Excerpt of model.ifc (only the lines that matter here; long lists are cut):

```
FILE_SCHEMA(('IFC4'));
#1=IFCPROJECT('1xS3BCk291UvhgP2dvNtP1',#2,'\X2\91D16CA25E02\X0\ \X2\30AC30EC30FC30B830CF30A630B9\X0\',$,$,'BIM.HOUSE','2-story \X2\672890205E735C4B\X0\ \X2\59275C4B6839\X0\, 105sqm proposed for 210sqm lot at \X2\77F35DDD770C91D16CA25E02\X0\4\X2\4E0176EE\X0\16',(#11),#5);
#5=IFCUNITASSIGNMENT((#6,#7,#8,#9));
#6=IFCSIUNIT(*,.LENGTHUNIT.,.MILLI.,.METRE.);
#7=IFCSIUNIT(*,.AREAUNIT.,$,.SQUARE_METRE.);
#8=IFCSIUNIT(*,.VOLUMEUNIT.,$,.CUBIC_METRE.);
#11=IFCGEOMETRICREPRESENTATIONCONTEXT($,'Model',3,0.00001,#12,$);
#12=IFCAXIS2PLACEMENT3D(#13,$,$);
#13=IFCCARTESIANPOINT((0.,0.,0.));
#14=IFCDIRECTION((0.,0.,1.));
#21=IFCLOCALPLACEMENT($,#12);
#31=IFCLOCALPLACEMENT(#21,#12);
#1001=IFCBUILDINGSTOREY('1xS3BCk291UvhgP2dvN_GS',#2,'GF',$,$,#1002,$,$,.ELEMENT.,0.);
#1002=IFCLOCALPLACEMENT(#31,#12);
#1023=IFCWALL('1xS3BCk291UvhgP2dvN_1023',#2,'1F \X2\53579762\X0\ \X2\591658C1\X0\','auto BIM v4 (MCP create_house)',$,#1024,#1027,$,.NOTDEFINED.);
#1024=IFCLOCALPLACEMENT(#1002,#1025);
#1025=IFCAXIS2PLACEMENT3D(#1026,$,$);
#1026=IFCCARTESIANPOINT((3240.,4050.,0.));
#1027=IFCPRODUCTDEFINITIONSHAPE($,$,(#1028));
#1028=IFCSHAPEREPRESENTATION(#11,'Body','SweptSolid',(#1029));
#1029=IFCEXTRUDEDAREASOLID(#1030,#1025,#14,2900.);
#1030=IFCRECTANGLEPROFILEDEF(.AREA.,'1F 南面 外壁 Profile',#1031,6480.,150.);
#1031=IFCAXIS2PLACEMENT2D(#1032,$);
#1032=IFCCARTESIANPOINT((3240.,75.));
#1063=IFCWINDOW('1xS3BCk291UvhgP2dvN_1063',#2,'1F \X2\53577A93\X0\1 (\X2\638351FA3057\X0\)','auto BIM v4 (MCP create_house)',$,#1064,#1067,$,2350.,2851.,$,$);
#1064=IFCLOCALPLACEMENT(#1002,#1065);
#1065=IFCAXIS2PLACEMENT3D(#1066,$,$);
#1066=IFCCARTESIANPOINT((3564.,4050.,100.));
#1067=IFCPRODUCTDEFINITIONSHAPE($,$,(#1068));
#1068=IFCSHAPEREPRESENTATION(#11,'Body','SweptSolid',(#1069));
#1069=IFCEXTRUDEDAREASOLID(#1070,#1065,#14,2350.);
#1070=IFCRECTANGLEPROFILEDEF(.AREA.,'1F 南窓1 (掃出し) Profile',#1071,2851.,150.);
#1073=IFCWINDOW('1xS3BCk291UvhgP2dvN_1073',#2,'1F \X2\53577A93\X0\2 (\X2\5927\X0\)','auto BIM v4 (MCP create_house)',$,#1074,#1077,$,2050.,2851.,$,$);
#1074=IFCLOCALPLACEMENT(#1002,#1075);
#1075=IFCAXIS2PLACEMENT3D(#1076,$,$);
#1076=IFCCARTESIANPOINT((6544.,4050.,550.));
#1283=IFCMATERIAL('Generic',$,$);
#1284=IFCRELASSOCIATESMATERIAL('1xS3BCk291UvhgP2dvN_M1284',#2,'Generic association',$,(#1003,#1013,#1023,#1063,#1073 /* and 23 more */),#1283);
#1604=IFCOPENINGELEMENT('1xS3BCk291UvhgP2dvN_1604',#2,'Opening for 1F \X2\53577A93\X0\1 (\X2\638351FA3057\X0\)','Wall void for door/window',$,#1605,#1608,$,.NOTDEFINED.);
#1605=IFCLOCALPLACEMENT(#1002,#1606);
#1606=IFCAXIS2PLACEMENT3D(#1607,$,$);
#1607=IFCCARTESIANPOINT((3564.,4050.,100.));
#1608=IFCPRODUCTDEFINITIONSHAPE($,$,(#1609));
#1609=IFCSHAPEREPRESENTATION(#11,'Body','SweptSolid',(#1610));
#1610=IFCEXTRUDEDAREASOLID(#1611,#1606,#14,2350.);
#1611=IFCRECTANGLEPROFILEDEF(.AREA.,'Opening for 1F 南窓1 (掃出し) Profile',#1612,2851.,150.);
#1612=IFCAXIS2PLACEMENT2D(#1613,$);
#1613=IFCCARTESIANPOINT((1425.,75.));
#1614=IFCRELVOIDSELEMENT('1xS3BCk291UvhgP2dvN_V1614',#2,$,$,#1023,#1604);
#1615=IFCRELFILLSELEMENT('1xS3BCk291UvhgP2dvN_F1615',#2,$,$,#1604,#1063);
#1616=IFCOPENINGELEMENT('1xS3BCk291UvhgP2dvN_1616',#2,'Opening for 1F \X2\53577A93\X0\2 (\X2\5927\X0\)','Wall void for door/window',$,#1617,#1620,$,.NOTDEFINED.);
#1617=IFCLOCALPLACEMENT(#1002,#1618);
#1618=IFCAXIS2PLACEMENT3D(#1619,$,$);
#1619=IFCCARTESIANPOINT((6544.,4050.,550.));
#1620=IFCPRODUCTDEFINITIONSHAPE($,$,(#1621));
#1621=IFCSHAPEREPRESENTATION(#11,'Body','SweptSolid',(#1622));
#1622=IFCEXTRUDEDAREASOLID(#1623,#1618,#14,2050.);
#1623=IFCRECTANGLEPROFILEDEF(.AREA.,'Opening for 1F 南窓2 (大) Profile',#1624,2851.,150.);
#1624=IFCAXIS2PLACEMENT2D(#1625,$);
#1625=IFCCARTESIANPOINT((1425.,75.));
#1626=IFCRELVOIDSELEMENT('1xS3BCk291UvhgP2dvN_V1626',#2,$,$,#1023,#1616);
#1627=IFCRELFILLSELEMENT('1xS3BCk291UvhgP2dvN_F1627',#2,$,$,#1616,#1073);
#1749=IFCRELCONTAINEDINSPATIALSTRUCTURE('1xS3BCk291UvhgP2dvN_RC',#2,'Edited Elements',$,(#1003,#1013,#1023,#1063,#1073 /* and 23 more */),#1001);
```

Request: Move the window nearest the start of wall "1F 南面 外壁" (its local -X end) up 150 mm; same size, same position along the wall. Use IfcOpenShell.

```python
import numpy as np
import ifcopenshell
import ifcopenshell.api.geometry
import ifcopenshell.util.placement
import ifcopenshell.util.unit

model = ifcopenshell.open("model.ifc")
unit_scale = ifcopenshell.util.unit.calculate_unit_scale(model)

window = model.by_id(1063)
opening = window.FillsVoids[0].RelatingOpeningElement
dz = 0.15 / unit_scale

shift = np.array([0.0, 0.0, dz])
# The window is not placed relative to its opening, so move both.
for product in (opening, window):
    matrix = ifcopenshell.util.placement.get_local_placement(product.ObjectPlacement)
    matrix[:3, 3] += shift
    ifcopenshell.api.geometry.edit_object_placement(model, product=product, matrix=matrix, is_si=False)

print(f"moved by {dz * unit_scale:+.3f} m")

model.write("model_rev.ifc")
```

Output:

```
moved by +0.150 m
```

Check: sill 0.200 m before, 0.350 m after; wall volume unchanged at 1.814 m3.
